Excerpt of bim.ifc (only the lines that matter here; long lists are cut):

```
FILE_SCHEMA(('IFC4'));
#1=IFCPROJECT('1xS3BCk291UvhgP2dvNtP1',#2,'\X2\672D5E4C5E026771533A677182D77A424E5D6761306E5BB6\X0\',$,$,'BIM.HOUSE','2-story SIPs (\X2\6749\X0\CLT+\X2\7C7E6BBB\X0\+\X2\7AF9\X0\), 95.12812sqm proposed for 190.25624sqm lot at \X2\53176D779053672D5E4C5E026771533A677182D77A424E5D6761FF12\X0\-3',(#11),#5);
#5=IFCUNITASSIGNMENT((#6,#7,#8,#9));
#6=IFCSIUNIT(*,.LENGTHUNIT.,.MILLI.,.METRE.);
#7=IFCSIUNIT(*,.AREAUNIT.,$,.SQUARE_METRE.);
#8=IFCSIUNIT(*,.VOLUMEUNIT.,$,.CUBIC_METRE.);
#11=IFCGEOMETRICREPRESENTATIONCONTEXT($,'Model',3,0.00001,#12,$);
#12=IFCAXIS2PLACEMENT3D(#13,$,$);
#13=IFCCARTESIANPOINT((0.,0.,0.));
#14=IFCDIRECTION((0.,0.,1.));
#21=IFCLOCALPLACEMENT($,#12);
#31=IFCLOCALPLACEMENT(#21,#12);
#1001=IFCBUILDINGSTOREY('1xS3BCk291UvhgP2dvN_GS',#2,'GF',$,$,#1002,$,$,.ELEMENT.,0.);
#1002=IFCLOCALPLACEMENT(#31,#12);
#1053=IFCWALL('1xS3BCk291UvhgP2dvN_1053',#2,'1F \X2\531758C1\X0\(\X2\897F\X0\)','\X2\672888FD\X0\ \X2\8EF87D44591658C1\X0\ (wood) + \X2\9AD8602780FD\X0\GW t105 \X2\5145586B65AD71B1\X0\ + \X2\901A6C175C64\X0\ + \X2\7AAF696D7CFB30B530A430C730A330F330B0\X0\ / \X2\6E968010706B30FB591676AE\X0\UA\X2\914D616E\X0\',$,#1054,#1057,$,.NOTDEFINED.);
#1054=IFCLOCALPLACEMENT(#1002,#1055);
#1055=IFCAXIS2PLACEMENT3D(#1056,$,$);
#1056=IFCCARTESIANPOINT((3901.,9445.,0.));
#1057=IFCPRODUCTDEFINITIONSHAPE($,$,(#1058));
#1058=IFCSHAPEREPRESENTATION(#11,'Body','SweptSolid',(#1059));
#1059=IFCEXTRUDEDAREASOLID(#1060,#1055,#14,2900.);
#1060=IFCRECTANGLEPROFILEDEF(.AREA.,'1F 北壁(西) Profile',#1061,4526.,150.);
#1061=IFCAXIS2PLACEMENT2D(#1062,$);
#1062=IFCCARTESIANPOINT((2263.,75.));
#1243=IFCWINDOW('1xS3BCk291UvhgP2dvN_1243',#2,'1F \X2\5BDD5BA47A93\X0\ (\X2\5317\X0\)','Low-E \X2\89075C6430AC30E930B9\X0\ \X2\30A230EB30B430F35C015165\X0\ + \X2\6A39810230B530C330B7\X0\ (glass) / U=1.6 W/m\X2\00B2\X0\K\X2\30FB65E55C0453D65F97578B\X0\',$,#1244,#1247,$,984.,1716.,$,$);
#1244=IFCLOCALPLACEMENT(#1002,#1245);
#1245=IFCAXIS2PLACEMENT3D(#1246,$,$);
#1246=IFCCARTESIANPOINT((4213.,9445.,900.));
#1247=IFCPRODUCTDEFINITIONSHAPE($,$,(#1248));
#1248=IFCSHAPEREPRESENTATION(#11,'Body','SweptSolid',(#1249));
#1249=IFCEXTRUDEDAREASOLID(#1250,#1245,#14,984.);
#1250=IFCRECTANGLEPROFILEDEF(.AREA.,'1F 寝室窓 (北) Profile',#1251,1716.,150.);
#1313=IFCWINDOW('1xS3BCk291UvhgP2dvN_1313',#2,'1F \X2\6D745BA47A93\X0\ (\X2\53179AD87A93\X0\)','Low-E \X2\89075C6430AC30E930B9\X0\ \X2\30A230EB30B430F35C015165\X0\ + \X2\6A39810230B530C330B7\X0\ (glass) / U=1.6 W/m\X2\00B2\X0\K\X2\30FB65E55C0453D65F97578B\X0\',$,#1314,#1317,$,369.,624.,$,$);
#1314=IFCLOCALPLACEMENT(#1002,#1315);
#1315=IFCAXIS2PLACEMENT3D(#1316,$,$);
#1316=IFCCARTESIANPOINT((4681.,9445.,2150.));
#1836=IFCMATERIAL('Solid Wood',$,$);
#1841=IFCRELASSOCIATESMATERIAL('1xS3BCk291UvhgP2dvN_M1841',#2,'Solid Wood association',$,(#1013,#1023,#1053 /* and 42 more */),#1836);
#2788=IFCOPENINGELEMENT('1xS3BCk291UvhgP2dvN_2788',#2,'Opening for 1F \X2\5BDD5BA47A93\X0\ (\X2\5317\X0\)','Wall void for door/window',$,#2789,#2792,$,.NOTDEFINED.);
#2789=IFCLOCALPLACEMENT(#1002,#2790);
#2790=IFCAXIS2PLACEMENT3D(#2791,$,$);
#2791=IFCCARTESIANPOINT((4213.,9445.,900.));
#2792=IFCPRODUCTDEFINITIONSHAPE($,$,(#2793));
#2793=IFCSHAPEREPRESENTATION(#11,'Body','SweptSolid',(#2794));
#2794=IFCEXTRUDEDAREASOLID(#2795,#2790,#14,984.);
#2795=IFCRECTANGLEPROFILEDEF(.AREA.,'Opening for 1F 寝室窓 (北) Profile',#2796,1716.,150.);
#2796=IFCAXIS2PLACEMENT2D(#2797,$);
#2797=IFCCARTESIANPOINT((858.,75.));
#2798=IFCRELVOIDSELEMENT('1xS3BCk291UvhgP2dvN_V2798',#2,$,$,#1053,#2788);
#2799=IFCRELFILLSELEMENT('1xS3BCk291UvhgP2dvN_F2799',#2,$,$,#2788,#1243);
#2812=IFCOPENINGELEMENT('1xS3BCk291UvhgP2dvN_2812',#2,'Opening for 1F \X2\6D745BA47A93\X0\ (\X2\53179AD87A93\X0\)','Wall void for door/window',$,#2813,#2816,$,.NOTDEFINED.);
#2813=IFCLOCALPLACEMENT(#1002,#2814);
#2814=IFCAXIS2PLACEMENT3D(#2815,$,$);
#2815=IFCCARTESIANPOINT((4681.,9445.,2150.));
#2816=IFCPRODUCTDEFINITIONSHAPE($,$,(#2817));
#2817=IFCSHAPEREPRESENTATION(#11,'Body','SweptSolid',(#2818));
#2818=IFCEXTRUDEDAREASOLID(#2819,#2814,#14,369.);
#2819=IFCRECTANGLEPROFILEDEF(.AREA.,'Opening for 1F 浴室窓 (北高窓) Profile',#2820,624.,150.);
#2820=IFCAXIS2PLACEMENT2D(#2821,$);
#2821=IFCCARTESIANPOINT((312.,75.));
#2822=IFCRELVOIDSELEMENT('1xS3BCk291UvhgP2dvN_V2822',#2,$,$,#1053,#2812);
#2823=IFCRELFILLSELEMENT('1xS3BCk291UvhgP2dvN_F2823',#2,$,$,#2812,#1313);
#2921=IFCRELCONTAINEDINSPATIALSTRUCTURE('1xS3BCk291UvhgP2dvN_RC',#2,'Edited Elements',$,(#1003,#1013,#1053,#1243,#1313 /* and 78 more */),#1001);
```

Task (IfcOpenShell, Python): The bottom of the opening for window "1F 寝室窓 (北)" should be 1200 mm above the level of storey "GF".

```python
import numpy as np
import ifcopenshell
import ifcopenshell.api.geometry
import ifcopenshell.geom
import ifcopenshell.util.element
import ifcopenshell.util.placement
import ifcopenshell.util.shape
import ifcopenshell.util.unit

model = ifcopenshell.open("bim.ifc")
unit_scale = ifcopenshell.util.unit.calculate_unit_scale(model)

window = model.by_guid("1xS3BCk291UvhgP2dvN_1243")
opening = window.FillsVoids[0].RelatingOpeningElement
storey = ifcopenshell.util.element.get_container(window, ifc_class="IfcBuildingStorey")
level = ifcopenshell.util.placement.get_local_placement(storey.ObjectPlacement)[2, 3]

# The opening's origin need not be at the sill, so measure its lowest point.
shape = ifcopenshell.geom.create_shape(ifcopenshell.geom.settings(), opening)
bottom = ifcopenshell.util.shape.get_shape_bottom_elevation(shape, shape.geometry) / unit_scale
dz = level + 1200.0 - bottom

shift = np.array([0.0, 0.0, dz])
# The window is not placed relative to its opening, so move both.
for product in (opening, window):
    matrix = ifcopenshell.util.placement.get_local_placement(product.ObjectPlacement)
    matrix[:3, 3] += shift
    ifcopenshell.api.geometry.edit_object_placement(model, product=product, matrix=matrix, is_si=False)

print(f"moved by {dz * unit_scale:+.3f} m")

model.write("bim_edited.ifc")
```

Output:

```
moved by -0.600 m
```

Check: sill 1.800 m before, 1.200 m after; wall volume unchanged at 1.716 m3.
